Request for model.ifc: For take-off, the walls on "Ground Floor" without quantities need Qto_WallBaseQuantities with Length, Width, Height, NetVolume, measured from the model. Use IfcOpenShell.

First a look at what the model holds.

```python
import ifcopenshell
import ifcopenshell.util.element
import ifcopenshell.util.unit

model = ifcopenshell.open("model.ifc")
print(model.schema)
for unit_type in ("LENGTHUNIT", "AREAUNIT", "VOLUMEUNIT"):
    print(unit_type, ifcopenshell.util.unit.calculate_unit_scale(model, unit_type))
storey = next(s for s in model.by_type("IfcBuildingStorey") if s.Name == "Ground Floor")
walls = [e for e in ifcopenshell.util.element.get_decomposition(storey) if e.is_a("IfcWall")]
for e in sorted(walls, key=lambda e: e.id()):
    print(e.id(), e.is_a(), e.Name, list(ifcopenshell.util.element.get_psets(e, qtos_only=True)), sep=" | ")
```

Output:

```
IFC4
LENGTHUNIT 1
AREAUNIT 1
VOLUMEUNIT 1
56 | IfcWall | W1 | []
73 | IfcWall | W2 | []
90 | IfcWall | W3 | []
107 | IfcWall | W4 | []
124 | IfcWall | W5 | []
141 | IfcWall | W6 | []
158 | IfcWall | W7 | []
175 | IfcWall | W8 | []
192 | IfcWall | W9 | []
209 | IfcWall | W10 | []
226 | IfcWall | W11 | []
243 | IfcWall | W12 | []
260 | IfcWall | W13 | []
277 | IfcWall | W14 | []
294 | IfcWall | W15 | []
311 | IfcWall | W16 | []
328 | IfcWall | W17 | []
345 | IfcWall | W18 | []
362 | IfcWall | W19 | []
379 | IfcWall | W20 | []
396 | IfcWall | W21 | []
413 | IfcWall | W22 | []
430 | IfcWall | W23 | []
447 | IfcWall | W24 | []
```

```python
import ifcopenshell
import ifcopenshell.api.pset
import ifcopenshell.geom
import ifcopenshell.util.element
import ifcopenshell.util.shape
import ifcopenshell.util.unit

model = ifcopenshell.open("model.ifc")
unit_scale = ifcopenshell.util.unit.calculate_unit_scale(model)
volume_scale = ifcopenshell.util.unit.calculate_unit_scale(model, "VOLUMEUNIT")
settings = ifcopenshell.geom.settings()

storey = next(s for s in model.by_type("IfcBuildingStorey") if s.Name == "Ground Floor")
walls = [e for e in ifcopenshell.util.element.get_decomposition(storey) if e.is_a("IfcWall")]

for e in sorted(walls, key=lambda e: e.id()):
    if ifcopenshell.util.element.get_psets(e, qtos_only=True, should_inherit=False):
        continue
    # Geometry comes back in metres, in the element's own axes.
    shape = ifcopenshell.geom.create_shape(settings, e)
    values = {
        "Length": ifcopenshell.util.shape.get_x(shape.geometry) / unit_scale,
        "Width": ifcopenshell.util.shape.get_y(shape.geometry) / unit_scale,
        "Height": ifcopenshell.util.shape.get_z(shape.geometry) / unit_scale,
        "NetVolume": ifcopenshell.util.shape.get_volume(shape.geometry) / volume_scale,
    }
    qto = ifcopenshell.api.pset.add_qto(model, product=e, name="Qto_WallBaseQuantities")
    ifcopenshell.api.pset.edit_qto(model, qto=qto, properties=values)
    print(e.id(), {k: round(v, 3) for k, v in values.items()})

model.write("model_rev.ifc")
```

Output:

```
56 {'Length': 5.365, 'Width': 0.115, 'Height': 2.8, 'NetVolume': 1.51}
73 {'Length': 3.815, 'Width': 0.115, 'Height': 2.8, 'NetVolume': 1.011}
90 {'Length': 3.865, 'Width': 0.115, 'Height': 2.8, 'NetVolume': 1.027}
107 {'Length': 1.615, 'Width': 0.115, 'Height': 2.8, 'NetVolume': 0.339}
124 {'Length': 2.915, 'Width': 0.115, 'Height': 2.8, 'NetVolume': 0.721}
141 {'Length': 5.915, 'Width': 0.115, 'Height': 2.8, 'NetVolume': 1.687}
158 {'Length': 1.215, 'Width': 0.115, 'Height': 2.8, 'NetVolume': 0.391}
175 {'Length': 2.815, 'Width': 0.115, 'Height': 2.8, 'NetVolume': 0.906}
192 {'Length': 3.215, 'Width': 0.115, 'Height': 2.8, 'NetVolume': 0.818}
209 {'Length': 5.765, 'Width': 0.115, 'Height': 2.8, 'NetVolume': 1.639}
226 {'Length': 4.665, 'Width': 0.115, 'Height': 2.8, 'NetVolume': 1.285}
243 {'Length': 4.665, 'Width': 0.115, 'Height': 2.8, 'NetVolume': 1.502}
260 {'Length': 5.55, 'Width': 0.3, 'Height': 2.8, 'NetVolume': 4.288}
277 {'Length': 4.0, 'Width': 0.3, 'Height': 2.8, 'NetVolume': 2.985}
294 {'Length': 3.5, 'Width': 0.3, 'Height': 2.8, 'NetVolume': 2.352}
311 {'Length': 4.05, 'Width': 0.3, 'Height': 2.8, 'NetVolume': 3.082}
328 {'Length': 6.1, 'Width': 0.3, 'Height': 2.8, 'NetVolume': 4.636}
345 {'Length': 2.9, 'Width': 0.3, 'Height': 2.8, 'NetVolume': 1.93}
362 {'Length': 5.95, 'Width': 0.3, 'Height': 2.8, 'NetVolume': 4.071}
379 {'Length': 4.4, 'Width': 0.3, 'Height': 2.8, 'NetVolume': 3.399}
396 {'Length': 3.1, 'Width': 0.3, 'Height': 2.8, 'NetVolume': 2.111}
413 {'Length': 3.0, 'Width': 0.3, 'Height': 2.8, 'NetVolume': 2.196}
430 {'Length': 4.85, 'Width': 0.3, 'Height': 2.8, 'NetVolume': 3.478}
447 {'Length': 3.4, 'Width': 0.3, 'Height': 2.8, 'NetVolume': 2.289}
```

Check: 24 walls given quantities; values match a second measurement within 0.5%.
